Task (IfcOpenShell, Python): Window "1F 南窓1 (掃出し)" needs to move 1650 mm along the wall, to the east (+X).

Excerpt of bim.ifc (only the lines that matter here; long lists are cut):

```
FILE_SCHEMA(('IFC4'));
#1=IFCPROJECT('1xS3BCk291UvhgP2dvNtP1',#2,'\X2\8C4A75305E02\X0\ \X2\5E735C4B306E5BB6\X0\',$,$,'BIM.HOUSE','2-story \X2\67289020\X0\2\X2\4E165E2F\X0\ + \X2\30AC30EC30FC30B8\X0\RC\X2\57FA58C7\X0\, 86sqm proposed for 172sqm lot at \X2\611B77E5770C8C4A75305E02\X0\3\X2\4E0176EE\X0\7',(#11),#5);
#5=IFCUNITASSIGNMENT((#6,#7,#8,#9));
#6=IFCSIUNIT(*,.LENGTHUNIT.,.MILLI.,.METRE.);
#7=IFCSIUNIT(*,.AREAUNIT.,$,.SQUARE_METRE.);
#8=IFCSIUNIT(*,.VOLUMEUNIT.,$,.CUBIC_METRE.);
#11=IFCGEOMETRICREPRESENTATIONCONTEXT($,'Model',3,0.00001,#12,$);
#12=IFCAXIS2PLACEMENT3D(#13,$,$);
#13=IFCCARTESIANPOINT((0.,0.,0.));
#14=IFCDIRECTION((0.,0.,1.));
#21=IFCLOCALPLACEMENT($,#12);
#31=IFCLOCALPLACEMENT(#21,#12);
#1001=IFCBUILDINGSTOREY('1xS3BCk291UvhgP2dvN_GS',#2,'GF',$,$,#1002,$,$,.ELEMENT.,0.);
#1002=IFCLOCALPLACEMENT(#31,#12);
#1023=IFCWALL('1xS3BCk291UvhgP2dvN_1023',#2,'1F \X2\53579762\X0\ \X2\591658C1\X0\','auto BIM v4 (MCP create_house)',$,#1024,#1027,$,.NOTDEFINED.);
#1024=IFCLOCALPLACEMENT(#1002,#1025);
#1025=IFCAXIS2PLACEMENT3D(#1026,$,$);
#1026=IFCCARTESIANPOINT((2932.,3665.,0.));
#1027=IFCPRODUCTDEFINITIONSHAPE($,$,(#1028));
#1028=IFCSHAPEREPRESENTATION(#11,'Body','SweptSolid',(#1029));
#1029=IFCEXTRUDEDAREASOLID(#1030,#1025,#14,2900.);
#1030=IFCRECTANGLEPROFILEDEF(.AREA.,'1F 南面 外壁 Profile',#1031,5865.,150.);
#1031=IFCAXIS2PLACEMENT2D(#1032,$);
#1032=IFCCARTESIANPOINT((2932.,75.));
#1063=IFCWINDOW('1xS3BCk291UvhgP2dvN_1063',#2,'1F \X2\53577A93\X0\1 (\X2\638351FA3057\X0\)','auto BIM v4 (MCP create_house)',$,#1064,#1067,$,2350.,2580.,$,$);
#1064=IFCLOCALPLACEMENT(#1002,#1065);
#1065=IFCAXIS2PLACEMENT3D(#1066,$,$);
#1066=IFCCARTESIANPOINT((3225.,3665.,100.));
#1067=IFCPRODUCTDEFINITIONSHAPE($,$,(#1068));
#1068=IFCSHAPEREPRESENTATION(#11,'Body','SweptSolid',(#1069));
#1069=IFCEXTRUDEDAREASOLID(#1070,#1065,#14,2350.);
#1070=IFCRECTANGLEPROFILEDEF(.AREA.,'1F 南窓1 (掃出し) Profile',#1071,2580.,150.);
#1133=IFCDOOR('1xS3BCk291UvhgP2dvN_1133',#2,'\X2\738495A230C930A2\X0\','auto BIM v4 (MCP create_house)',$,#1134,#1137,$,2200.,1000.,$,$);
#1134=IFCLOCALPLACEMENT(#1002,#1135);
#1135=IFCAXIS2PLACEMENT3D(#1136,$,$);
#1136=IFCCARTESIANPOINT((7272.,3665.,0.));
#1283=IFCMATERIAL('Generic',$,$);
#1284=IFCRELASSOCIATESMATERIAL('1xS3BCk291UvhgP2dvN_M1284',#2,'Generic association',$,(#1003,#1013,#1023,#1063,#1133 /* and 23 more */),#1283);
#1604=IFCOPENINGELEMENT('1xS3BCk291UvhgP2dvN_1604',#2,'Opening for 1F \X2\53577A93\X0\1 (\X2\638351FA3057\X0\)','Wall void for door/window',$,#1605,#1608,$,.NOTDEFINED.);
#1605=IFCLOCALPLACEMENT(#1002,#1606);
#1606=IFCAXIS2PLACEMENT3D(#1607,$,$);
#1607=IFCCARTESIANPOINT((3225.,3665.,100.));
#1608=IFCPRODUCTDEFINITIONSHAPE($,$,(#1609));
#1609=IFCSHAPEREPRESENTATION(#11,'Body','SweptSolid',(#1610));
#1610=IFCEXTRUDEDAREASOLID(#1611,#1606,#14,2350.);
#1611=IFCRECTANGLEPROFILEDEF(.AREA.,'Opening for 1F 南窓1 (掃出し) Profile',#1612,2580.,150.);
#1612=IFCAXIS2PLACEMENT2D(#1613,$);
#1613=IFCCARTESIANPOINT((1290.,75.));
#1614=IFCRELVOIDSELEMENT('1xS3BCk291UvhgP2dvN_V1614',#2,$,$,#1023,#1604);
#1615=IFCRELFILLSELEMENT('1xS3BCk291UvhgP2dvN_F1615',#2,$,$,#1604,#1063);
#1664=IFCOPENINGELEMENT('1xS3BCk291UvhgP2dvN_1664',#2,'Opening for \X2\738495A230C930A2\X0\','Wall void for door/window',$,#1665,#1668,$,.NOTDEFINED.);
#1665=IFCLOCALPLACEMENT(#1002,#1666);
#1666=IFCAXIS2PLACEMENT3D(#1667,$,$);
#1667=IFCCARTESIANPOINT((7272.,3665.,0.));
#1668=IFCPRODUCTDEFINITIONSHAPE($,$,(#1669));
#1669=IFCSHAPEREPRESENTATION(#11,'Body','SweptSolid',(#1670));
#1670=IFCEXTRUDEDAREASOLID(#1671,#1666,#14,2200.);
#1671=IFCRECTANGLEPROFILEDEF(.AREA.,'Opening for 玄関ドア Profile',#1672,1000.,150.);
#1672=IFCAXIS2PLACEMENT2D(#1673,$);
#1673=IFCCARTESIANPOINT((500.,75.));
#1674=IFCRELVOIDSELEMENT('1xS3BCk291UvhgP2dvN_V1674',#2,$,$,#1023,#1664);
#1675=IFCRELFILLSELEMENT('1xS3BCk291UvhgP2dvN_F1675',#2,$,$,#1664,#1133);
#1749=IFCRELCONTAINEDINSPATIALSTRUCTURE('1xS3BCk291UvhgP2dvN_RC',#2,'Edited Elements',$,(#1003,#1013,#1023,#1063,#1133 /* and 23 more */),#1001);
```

```python
import ifcopenshell
import ifcopenshell.api.geometry
import ifcopenshell.util.placement

model = ifcopenshell.open("bim.ifc")

window = model.by_guid("1xS3BCk291UvhgP2dvN_1063")
opening = window.FillsVoids[0].RelatingOpeningElement
wall = opening.VoidsElements[0].RelatingBuildingElement

wall_matrix = ifcopenshell.util.placement.get_local_placement(wall.ObjectPlacement)
shift = wall_matrix[:3, 0] * 1650.0
before = ifcopenshell.util.placement.get_local_placement(window.ObjectPlacement)[:3, 3].copy()

# The window is not placed relative to its opening, so move both.
for product in (opening, window):
    matrix = ifcopenshell.util.placement.get_local_placement(product.ObjectPlacement)
    matrix[:3, 3] += shift
    ifcopenshell.api.geometry.edit_object_placement(model, product=product, matrix=matrix, is_si=False)

after = ifcopenshell.util.placement.get_local_placement(window.ObjectPlacement)[:3, 3]
print("window moved by", (after - before).round(3) + 0.0)

model.write("bim_v2.ifc")
```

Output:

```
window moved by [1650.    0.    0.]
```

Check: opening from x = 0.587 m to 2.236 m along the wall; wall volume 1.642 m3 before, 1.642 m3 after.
